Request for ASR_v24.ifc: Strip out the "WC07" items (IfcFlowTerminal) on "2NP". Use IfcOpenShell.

First a look at what the model holds.

```python
import ifcopenshell
import ifcopenshell.util.element

model = ifcopenshell.open("ASR_v24.ifc")
print(model.schema)
storey = next(s for s in model.by_type("IfcBuildingStorey") if s.Name == "2NP")
terminals = [e for e in ifcopenshell.util.element.get_decomposition(storey) if e.is_a("IfcFlowTerminal")]
seen = {}
for e in terminals:
    element_type = ifcopenshell.util.element.get_type(e)
    name = element_type.Name if element_type not in (None, e) else None
    seen[name] = seen.get(name, 0) + 1
for name, count in sorted(seen.items(), key=str):
    print(count, "x", name)
```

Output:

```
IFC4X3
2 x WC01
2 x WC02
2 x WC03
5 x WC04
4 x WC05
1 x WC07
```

```python
import ifcopenshell
import ifcopenshell.api.root
import ifcopenshell.util.element

model = ifcopenshell.open("ASR_v24.ifc")

storey = next(s for s in model.by_type("IfcBuildingStorey") if s.Name == "2NP")
terminals = [e for e in ifcopenshell.util.element.get_decomposition(storey) if e.is_a("IfcFlowTerminal")]
targets = [e for e in terminals if (t := ifcopenshell.util.element.get_type(e)) not in (None, e) and t.Name == "WC07"]

for e in targets:
    ifcopenshell.api.root.remove_product(model, product=e)
print(len(targets), "removed")

model.write("ASR_v24_updated.ifc")
```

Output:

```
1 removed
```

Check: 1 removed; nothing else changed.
